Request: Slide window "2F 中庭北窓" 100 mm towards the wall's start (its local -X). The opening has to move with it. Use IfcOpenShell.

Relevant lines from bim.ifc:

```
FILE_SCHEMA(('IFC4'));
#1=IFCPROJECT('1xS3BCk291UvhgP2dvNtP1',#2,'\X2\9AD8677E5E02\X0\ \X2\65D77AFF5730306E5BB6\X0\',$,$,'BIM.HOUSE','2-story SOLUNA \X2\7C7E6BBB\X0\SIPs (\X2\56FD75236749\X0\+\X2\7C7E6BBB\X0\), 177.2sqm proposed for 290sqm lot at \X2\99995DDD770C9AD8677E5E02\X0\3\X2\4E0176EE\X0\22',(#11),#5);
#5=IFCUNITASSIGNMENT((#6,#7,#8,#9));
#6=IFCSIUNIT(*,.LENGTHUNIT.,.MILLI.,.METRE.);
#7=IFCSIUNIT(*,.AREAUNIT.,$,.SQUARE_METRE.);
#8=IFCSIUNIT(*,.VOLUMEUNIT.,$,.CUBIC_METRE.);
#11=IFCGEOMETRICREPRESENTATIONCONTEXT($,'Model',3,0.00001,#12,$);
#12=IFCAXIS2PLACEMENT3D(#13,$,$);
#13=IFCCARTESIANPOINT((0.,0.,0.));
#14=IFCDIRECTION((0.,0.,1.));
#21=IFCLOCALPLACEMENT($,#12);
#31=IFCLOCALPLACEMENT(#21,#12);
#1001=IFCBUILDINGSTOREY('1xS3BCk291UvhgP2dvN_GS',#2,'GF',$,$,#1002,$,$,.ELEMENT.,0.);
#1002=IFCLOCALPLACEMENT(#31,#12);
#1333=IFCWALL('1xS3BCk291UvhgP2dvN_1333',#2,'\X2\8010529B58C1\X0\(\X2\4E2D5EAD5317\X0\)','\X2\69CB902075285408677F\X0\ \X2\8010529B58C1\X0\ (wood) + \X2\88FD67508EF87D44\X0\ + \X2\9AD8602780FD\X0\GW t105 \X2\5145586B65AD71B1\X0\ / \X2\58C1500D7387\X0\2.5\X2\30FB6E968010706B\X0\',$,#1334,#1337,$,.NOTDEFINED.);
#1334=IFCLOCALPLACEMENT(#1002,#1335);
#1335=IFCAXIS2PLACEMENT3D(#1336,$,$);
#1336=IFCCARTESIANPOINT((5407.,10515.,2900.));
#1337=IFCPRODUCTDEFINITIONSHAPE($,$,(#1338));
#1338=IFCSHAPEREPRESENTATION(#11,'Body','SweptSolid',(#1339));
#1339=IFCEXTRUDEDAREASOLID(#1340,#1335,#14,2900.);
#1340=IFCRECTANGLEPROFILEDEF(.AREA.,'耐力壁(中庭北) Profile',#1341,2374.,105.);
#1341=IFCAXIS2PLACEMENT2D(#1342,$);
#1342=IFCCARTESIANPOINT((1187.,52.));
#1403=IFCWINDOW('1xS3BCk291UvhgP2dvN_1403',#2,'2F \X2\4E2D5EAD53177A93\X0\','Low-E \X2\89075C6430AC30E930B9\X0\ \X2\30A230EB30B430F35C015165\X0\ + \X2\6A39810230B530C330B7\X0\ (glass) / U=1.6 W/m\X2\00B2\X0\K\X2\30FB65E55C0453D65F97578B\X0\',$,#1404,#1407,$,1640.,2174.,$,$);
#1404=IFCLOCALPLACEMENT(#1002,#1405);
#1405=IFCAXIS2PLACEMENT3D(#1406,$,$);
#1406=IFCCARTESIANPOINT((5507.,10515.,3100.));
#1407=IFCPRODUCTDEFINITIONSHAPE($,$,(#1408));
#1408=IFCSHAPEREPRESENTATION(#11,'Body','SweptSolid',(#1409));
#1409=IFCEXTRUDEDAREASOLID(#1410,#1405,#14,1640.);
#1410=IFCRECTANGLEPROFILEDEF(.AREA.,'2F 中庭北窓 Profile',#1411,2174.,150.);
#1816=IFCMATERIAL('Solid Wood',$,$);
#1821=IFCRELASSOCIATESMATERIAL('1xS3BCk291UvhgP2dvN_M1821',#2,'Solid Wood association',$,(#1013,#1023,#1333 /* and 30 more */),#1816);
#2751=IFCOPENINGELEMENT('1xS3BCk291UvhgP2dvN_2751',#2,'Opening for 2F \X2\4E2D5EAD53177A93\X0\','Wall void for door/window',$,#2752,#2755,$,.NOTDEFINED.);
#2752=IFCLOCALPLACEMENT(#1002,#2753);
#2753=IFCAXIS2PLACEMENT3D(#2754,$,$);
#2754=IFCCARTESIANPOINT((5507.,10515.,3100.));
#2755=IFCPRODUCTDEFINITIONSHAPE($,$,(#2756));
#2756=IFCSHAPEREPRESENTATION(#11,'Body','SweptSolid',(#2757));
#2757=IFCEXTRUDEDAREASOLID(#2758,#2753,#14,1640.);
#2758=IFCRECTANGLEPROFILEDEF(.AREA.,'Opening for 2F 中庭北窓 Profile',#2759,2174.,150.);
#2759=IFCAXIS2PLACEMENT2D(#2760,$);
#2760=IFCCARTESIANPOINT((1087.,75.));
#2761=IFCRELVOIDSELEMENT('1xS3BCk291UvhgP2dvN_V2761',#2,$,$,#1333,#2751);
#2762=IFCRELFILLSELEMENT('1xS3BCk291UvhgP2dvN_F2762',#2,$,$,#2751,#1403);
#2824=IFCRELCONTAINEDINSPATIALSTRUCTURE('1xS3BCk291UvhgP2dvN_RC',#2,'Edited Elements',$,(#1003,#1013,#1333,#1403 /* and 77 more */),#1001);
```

```python
import ifcopenshell
import ifcopenshell.api.geometry
import ifcopenshell.util.placement
import ifcopenshell.util.unit

model = ifcopenshell.open("bim.ifc")
unit_scale = ifcopenshell.util.unit.calculate_unit_scale(model)

window = model.by_guid("1xS3BCk291UvhgP2dvN_1403")
opening = window.FillsVoids[0].RelatingOpeningElement
wall = opening.VoidsElements[0].RelatingBuildingElement

wall_matrix = ifcopenshell.util.placement.get_local_placement(wall.ObjectPlacement)
shift = wall_matrix[:3, 0] * -0.1 / unit_scale
before = ifcopenshell.util.placement.get_local_placement(window.ObjectPlacement)[:3, 3].copy()

# The window is not placed relative to its opening, so move both.
for product in (opening, window):
    matrix = ifcopenshell.util.placement.get_local_placement(product.ObjectPlacement)
    matrix[:3, 3] += shift
    ifcopenshell.api.geometry.edit_object_placement(model, product=product, matrix=matrix, is_si=False)

after = ifcopenshell.util.placement.get_local_placement(window.ObjectPlacement)[:3, 3]
print("window moved by", (after - before).round(3) + 0.0)

model.write("bim_rev.ifc")
```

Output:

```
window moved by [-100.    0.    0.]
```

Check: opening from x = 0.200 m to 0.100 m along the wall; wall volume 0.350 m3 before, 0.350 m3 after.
